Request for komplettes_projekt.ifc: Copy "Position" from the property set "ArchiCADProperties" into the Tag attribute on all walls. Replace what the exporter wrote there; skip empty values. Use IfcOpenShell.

First a look at what the model holds.

```python
import ifcopenshell
import ifcopenshell.util.element

model = ifcopenshell.open("komplettes_projekt.ifc")
print(model.schema)
walls = model.by_type("IfcWall")
print(len(walls), "walls")
for e in walls[:8]:
    source = ifcopenshell.util.element.get_pset(e, "ArchiCADProperties", "Position")
    target = e.Tag
    print(e.id(), repr(source), repr(target), sep=" | ")
```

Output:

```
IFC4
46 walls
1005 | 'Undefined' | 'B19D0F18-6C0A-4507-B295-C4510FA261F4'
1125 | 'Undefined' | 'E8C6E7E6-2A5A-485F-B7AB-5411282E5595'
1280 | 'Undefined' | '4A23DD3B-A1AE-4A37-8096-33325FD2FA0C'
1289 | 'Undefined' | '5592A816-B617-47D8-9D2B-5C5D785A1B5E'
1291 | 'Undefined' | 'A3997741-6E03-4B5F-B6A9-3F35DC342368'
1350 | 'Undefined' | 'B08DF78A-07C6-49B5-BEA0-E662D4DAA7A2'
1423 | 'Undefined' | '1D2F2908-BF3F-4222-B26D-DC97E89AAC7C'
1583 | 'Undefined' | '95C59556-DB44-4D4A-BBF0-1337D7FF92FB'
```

```python
import ifcopenshell
import ifcopenshell.util.element

model = ifcopenshell.open("komplettes_projekt.ifc")

count = 0
for e in model.by_type("IfcWall"):
    value = ifcopenshell.util.element.get_pset(e, "ArchiCADProperties", "Position")
    current = e.Tag
    if not value or not value.strip() or current == value:
        continue
    e.Tag = value
    count += 1

print(count, "walls updated")

model.write("komplettes_projekt-out.ifc")
```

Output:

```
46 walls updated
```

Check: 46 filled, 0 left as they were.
